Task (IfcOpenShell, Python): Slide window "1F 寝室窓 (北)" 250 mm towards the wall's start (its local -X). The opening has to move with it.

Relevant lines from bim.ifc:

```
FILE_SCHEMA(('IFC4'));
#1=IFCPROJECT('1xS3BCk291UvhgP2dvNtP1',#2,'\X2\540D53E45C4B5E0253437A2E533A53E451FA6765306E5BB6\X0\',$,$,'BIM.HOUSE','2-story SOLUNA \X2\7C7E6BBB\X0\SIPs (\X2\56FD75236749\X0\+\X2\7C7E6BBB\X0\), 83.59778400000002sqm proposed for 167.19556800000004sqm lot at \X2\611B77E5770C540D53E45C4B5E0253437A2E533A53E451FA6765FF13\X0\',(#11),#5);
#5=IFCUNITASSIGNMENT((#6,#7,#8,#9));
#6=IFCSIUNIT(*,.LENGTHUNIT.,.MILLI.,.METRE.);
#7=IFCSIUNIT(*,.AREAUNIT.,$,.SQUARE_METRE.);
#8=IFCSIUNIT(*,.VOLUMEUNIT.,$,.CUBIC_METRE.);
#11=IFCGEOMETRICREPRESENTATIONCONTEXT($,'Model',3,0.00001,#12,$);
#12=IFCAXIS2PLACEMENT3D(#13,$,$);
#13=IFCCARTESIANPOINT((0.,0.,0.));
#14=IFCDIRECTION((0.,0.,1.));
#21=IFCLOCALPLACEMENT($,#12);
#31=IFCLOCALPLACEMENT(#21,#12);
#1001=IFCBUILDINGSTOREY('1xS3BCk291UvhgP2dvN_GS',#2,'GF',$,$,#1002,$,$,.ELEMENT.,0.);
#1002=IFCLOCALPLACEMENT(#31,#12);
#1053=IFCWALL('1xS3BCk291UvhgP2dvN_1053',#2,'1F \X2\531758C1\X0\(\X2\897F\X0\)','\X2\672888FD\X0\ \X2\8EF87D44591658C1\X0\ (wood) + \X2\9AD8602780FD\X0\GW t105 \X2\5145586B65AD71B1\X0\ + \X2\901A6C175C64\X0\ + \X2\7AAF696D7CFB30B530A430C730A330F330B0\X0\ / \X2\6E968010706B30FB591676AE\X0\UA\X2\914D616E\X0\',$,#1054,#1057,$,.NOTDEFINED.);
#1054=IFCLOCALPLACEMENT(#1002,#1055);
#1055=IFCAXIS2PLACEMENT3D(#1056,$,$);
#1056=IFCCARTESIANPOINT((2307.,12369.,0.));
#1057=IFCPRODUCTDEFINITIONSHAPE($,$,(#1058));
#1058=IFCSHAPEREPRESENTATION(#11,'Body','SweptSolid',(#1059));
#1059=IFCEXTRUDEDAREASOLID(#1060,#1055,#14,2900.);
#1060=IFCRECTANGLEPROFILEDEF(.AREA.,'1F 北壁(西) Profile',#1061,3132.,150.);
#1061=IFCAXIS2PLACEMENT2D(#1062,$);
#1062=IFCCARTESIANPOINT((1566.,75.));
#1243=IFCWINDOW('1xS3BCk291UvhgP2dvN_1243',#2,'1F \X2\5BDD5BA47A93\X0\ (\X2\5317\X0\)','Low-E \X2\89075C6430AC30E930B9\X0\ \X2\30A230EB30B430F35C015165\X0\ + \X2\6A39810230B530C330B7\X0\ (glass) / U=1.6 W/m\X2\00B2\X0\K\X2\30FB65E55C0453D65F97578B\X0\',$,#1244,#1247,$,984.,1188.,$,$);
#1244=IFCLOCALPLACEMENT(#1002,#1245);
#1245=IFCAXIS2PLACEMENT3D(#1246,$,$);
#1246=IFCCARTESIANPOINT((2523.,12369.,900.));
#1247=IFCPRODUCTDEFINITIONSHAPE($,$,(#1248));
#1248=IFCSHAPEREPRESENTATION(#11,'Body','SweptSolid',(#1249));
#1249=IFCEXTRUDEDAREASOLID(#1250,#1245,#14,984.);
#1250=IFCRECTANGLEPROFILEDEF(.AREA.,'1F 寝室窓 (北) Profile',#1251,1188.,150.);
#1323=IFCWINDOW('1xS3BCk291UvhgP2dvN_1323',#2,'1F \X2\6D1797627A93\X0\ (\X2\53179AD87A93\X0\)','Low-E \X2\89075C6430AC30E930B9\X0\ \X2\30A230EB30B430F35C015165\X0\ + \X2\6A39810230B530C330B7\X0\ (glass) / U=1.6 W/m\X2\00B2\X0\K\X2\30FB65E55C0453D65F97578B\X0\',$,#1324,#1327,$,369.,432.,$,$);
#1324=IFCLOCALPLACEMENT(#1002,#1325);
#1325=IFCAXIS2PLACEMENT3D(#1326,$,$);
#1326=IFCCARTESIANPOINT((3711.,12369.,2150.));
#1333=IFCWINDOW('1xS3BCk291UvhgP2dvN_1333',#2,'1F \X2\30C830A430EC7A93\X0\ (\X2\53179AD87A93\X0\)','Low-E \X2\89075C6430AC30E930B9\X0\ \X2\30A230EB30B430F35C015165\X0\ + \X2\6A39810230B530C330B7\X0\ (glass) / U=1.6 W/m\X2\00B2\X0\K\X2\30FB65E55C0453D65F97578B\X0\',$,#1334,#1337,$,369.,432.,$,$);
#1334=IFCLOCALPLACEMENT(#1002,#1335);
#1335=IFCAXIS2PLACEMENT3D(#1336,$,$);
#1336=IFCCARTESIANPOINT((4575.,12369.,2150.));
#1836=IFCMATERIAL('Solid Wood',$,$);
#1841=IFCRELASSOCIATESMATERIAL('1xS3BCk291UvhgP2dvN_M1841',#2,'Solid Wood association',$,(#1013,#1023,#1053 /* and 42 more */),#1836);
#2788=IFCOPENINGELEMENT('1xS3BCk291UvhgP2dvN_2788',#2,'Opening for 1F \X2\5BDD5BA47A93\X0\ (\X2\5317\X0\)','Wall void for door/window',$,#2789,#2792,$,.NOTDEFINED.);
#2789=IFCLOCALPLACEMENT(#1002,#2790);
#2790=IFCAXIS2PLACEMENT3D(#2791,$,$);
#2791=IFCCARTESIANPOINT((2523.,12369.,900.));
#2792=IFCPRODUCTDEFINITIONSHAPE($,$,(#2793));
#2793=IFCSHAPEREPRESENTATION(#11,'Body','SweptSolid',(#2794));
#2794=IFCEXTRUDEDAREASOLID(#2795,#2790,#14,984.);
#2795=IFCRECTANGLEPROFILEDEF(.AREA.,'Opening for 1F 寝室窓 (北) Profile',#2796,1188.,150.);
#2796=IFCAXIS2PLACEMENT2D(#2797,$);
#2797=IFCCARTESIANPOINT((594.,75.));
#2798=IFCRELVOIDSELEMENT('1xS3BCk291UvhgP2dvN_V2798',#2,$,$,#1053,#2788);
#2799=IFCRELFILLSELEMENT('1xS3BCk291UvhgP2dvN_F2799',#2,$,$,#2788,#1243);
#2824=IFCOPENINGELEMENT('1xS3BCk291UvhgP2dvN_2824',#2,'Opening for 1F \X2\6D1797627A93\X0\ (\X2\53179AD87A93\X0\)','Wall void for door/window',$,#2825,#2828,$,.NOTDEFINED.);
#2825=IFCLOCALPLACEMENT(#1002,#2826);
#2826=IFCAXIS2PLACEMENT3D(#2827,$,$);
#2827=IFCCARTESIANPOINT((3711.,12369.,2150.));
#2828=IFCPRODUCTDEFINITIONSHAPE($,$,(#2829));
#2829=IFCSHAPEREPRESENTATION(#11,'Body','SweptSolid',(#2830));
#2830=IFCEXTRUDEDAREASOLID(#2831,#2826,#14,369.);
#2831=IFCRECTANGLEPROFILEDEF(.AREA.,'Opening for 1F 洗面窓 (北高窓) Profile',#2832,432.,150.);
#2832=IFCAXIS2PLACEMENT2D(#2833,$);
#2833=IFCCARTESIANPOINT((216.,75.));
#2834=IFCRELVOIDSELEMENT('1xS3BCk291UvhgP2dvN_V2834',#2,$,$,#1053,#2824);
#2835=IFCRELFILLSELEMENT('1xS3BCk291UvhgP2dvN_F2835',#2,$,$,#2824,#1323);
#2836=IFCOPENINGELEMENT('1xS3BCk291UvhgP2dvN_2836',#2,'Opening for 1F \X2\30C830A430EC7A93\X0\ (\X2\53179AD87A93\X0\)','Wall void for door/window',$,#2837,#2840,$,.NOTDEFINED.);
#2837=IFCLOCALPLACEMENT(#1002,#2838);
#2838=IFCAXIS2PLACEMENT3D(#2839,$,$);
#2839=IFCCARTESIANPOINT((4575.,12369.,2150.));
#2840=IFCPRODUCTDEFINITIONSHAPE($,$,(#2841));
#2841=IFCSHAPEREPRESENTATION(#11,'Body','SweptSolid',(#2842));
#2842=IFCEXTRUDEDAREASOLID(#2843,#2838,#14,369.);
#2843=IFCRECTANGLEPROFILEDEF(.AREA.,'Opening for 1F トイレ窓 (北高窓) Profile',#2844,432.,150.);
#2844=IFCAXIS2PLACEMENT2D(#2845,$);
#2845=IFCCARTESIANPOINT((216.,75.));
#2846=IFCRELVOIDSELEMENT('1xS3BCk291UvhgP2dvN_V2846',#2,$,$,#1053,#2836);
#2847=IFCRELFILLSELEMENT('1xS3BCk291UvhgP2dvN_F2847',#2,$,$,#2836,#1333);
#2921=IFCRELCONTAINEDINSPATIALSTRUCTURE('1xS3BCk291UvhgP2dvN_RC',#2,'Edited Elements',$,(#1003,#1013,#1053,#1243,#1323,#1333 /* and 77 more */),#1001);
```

```python
import ifcopenshell
import ifcopenshell.api.geometry
import ifcopenshell.util.placement
import ifcopenshell.util.unit

model = ifcopenshell.open("bim.ifc")
unit_scale = ifcopenshell.util.unit.calculate_unit_scale(model)

window = model.by_guid("1xS3BCk291UvhgP2dvN_1243")
opening = window.FillsVoids[0].RelatingOpeningElement
wall = opening.VoidsElements[0].RelatingBuildingElement

wall_matrix = ifcopenshell.util.placement.get_local_placement(wall.ObjectPlacement)
shift = wall_matrix[:3, 0] * -0.25 / unit_scale
before = ifcopenshell.util.placement.get_local_placement(window.ObjectPlacement)[:3, 3].copy()

# The window is not placed relative to its opening, so move both.
for product in (opening, window):
    matrix = ifcopenshell.util.placement.get_local_placement(product.ObjectPlacement)
    matrix[:3, 3] += shift
    ifcopenshell.api.geometry.edit_object_placement(model, product=product, matrix=matrix, is_si=False)

after = ifcopenshell.util.placement.get_local_placement(window.ObjectPlacement)[:3, 3]
print("window moved by", (after - before).round(3) + 0.0)

model.write("bim_v2.ifc")
```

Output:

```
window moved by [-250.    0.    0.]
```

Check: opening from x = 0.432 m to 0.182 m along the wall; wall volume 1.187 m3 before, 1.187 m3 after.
